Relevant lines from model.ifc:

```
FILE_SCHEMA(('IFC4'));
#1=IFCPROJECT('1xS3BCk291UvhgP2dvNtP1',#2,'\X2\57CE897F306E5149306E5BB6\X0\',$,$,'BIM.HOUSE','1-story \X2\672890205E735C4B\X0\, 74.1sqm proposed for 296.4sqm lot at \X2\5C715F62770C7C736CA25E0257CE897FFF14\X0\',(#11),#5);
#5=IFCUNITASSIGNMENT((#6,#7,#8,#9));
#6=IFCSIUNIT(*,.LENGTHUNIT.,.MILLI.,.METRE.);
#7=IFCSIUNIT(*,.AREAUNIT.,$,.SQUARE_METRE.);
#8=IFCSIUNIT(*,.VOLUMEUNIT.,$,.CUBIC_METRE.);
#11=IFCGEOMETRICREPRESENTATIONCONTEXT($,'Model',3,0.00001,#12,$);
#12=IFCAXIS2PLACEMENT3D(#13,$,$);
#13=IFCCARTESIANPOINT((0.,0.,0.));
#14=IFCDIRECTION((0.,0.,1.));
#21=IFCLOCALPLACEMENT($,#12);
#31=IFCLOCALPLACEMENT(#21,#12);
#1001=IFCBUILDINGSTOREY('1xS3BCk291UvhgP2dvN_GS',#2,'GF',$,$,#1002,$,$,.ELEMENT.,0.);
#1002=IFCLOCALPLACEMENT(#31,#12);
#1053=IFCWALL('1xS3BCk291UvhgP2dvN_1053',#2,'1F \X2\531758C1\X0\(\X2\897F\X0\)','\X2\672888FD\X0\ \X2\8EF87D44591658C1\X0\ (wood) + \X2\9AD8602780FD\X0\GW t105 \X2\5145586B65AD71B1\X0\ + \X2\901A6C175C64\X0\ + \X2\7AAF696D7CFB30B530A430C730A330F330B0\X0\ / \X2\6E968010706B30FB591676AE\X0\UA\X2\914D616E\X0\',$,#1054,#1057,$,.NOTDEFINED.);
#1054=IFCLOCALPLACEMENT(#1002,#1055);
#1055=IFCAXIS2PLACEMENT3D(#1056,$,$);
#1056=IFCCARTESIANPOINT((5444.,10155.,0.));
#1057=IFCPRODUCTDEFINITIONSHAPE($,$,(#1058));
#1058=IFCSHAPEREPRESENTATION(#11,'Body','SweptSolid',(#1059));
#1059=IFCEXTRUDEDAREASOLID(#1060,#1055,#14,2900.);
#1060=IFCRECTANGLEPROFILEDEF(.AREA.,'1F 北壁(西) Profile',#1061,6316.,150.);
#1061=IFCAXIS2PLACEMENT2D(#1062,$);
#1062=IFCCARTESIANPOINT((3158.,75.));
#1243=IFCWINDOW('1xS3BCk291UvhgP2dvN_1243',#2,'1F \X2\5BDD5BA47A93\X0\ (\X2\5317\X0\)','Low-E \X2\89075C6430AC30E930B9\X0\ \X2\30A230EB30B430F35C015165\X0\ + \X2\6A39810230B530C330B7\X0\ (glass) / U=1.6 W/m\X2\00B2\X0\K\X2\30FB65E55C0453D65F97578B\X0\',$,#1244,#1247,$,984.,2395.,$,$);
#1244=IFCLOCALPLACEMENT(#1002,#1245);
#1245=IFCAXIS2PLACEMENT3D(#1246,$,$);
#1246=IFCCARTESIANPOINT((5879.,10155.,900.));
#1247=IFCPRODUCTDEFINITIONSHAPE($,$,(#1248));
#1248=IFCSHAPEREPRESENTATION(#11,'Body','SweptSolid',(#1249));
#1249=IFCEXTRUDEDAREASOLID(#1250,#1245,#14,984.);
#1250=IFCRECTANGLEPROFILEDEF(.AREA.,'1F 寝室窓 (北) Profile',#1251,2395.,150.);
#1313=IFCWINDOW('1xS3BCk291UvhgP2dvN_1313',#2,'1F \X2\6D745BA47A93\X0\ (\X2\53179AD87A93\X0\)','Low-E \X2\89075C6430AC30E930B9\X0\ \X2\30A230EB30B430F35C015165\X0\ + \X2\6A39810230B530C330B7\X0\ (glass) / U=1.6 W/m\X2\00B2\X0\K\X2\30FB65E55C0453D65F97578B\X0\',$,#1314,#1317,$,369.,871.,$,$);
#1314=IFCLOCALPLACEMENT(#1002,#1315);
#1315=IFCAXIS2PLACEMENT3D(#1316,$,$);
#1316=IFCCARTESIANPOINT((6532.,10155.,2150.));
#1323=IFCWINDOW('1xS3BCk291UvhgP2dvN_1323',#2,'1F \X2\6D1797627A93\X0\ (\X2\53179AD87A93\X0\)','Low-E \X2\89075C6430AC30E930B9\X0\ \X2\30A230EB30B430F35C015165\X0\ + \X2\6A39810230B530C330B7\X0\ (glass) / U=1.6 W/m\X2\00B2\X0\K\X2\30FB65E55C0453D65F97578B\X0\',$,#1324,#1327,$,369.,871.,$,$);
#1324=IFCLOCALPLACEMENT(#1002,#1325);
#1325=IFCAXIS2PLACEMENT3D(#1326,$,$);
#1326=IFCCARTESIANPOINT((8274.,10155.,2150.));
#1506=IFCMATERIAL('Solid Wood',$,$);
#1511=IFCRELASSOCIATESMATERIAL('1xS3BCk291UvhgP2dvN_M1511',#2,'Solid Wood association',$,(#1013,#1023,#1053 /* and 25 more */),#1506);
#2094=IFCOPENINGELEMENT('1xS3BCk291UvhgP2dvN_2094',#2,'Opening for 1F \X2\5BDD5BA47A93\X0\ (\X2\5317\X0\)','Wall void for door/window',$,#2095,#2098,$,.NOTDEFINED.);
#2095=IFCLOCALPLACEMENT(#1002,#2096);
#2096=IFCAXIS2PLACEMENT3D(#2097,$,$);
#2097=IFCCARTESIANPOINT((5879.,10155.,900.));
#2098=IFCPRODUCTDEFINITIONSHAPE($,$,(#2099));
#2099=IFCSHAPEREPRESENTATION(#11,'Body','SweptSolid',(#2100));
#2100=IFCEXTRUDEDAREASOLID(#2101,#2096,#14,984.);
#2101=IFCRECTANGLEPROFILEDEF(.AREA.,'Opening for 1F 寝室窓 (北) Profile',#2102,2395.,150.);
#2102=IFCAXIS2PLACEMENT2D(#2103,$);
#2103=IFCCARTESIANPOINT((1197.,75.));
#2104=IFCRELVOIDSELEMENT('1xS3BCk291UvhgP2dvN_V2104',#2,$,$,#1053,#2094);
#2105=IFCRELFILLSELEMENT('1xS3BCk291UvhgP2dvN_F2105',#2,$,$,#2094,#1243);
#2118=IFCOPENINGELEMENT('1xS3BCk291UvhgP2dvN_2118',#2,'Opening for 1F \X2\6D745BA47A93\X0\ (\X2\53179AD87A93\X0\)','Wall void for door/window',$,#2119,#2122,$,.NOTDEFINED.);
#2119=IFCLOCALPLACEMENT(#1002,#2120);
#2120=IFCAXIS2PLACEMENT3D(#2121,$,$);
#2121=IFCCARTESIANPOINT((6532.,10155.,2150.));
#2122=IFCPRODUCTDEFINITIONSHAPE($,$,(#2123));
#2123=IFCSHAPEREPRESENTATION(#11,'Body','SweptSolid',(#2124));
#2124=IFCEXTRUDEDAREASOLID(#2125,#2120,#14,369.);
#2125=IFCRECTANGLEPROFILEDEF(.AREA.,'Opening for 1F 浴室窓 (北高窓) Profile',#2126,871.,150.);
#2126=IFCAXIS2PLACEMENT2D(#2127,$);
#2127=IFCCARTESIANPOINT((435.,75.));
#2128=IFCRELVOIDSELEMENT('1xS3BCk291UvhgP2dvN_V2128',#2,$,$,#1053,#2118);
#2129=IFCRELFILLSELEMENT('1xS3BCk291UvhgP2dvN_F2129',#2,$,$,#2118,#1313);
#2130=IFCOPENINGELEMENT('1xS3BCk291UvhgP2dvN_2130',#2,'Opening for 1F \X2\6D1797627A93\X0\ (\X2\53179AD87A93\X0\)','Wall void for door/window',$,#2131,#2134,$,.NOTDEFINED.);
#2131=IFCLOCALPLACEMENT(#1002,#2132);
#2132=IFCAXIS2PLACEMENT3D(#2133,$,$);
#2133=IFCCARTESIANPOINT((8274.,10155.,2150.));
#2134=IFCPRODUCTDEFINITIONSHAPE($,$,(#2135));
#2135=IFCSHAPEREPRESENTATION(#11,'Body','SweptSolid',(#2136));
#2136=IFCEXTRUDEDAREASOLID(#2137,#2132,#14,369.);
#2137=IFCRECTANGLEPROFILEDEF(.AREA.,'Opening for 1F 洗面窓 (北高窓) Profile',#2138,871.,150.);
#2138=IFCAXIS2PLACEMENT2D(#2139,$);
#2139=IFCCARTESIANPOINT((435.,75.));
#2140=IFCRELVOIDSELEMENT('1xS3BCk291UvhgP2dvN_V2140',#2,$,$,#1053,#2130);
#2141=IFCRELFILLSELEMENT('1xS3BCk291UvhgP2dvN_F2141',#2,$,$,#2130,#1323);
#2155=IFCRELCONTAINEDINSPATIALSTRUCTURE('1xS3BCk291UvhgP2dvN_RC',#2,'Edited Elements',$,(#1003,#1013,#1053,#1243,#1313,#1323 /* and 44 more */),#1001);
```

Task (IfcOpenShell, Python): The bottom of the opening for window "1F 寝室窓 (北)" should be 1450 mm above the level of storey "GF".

```python
import numpy as np
import ifcopenshell
import ifcopenshell.api.geometry
import ifcopenshell.geom
import ifcopenshell.util.element
import ifcopenshell.util.placement
import ifcopenshell.util.shape
import ifcopenshell.util.unit

model = ifcopenshell.open("model.ifc")
unit_scale = ifcopenshell.util.unit.calculate_unit_scale(model)

window = model.by_guid("1xS3BCk291UvhgP2dvN_1243")
opening = window.FillsVoids[0].RelatingOpeningElement
storey = ifcopenshell.util.element.get_container(window, ifc_class="IfcBuildingStorey")
level = ifcopenshell.util.placement.get_local_placement(storey.ObjectPlacement)[2, 3]

# The opening's origin need not be at the sill, so measure its lowest point.
shape = ifcopenshell.geom.create_shape(ifcopenshell.geom.settings(), opening)
bottom = ifcopenshell.util.shape.get_shape_bottom_elevation(shape, shape.geometry) / unit_scale
dz = level + 1450.0 - bottom

shift = np.array([0.0, 0.0, dz])
# The window is not placed relative to its opening, so move both.
for product in (opening, window):
    matrix = ifcopenshell.util.placement.get_local_placement(product.ObjectPlacement)
    matrix[:3, 3] += shift
    ifcopenshell.api.geometry.edit_object_placement(model, product=product, matrix=matrix, is_si=False)

print(f"moved by {dz * unit_scale:+.3f} m")

model.write("model_rev.ifc")
```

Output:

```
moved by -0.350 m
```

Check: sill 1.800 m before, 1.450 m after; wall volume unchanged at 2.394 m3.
